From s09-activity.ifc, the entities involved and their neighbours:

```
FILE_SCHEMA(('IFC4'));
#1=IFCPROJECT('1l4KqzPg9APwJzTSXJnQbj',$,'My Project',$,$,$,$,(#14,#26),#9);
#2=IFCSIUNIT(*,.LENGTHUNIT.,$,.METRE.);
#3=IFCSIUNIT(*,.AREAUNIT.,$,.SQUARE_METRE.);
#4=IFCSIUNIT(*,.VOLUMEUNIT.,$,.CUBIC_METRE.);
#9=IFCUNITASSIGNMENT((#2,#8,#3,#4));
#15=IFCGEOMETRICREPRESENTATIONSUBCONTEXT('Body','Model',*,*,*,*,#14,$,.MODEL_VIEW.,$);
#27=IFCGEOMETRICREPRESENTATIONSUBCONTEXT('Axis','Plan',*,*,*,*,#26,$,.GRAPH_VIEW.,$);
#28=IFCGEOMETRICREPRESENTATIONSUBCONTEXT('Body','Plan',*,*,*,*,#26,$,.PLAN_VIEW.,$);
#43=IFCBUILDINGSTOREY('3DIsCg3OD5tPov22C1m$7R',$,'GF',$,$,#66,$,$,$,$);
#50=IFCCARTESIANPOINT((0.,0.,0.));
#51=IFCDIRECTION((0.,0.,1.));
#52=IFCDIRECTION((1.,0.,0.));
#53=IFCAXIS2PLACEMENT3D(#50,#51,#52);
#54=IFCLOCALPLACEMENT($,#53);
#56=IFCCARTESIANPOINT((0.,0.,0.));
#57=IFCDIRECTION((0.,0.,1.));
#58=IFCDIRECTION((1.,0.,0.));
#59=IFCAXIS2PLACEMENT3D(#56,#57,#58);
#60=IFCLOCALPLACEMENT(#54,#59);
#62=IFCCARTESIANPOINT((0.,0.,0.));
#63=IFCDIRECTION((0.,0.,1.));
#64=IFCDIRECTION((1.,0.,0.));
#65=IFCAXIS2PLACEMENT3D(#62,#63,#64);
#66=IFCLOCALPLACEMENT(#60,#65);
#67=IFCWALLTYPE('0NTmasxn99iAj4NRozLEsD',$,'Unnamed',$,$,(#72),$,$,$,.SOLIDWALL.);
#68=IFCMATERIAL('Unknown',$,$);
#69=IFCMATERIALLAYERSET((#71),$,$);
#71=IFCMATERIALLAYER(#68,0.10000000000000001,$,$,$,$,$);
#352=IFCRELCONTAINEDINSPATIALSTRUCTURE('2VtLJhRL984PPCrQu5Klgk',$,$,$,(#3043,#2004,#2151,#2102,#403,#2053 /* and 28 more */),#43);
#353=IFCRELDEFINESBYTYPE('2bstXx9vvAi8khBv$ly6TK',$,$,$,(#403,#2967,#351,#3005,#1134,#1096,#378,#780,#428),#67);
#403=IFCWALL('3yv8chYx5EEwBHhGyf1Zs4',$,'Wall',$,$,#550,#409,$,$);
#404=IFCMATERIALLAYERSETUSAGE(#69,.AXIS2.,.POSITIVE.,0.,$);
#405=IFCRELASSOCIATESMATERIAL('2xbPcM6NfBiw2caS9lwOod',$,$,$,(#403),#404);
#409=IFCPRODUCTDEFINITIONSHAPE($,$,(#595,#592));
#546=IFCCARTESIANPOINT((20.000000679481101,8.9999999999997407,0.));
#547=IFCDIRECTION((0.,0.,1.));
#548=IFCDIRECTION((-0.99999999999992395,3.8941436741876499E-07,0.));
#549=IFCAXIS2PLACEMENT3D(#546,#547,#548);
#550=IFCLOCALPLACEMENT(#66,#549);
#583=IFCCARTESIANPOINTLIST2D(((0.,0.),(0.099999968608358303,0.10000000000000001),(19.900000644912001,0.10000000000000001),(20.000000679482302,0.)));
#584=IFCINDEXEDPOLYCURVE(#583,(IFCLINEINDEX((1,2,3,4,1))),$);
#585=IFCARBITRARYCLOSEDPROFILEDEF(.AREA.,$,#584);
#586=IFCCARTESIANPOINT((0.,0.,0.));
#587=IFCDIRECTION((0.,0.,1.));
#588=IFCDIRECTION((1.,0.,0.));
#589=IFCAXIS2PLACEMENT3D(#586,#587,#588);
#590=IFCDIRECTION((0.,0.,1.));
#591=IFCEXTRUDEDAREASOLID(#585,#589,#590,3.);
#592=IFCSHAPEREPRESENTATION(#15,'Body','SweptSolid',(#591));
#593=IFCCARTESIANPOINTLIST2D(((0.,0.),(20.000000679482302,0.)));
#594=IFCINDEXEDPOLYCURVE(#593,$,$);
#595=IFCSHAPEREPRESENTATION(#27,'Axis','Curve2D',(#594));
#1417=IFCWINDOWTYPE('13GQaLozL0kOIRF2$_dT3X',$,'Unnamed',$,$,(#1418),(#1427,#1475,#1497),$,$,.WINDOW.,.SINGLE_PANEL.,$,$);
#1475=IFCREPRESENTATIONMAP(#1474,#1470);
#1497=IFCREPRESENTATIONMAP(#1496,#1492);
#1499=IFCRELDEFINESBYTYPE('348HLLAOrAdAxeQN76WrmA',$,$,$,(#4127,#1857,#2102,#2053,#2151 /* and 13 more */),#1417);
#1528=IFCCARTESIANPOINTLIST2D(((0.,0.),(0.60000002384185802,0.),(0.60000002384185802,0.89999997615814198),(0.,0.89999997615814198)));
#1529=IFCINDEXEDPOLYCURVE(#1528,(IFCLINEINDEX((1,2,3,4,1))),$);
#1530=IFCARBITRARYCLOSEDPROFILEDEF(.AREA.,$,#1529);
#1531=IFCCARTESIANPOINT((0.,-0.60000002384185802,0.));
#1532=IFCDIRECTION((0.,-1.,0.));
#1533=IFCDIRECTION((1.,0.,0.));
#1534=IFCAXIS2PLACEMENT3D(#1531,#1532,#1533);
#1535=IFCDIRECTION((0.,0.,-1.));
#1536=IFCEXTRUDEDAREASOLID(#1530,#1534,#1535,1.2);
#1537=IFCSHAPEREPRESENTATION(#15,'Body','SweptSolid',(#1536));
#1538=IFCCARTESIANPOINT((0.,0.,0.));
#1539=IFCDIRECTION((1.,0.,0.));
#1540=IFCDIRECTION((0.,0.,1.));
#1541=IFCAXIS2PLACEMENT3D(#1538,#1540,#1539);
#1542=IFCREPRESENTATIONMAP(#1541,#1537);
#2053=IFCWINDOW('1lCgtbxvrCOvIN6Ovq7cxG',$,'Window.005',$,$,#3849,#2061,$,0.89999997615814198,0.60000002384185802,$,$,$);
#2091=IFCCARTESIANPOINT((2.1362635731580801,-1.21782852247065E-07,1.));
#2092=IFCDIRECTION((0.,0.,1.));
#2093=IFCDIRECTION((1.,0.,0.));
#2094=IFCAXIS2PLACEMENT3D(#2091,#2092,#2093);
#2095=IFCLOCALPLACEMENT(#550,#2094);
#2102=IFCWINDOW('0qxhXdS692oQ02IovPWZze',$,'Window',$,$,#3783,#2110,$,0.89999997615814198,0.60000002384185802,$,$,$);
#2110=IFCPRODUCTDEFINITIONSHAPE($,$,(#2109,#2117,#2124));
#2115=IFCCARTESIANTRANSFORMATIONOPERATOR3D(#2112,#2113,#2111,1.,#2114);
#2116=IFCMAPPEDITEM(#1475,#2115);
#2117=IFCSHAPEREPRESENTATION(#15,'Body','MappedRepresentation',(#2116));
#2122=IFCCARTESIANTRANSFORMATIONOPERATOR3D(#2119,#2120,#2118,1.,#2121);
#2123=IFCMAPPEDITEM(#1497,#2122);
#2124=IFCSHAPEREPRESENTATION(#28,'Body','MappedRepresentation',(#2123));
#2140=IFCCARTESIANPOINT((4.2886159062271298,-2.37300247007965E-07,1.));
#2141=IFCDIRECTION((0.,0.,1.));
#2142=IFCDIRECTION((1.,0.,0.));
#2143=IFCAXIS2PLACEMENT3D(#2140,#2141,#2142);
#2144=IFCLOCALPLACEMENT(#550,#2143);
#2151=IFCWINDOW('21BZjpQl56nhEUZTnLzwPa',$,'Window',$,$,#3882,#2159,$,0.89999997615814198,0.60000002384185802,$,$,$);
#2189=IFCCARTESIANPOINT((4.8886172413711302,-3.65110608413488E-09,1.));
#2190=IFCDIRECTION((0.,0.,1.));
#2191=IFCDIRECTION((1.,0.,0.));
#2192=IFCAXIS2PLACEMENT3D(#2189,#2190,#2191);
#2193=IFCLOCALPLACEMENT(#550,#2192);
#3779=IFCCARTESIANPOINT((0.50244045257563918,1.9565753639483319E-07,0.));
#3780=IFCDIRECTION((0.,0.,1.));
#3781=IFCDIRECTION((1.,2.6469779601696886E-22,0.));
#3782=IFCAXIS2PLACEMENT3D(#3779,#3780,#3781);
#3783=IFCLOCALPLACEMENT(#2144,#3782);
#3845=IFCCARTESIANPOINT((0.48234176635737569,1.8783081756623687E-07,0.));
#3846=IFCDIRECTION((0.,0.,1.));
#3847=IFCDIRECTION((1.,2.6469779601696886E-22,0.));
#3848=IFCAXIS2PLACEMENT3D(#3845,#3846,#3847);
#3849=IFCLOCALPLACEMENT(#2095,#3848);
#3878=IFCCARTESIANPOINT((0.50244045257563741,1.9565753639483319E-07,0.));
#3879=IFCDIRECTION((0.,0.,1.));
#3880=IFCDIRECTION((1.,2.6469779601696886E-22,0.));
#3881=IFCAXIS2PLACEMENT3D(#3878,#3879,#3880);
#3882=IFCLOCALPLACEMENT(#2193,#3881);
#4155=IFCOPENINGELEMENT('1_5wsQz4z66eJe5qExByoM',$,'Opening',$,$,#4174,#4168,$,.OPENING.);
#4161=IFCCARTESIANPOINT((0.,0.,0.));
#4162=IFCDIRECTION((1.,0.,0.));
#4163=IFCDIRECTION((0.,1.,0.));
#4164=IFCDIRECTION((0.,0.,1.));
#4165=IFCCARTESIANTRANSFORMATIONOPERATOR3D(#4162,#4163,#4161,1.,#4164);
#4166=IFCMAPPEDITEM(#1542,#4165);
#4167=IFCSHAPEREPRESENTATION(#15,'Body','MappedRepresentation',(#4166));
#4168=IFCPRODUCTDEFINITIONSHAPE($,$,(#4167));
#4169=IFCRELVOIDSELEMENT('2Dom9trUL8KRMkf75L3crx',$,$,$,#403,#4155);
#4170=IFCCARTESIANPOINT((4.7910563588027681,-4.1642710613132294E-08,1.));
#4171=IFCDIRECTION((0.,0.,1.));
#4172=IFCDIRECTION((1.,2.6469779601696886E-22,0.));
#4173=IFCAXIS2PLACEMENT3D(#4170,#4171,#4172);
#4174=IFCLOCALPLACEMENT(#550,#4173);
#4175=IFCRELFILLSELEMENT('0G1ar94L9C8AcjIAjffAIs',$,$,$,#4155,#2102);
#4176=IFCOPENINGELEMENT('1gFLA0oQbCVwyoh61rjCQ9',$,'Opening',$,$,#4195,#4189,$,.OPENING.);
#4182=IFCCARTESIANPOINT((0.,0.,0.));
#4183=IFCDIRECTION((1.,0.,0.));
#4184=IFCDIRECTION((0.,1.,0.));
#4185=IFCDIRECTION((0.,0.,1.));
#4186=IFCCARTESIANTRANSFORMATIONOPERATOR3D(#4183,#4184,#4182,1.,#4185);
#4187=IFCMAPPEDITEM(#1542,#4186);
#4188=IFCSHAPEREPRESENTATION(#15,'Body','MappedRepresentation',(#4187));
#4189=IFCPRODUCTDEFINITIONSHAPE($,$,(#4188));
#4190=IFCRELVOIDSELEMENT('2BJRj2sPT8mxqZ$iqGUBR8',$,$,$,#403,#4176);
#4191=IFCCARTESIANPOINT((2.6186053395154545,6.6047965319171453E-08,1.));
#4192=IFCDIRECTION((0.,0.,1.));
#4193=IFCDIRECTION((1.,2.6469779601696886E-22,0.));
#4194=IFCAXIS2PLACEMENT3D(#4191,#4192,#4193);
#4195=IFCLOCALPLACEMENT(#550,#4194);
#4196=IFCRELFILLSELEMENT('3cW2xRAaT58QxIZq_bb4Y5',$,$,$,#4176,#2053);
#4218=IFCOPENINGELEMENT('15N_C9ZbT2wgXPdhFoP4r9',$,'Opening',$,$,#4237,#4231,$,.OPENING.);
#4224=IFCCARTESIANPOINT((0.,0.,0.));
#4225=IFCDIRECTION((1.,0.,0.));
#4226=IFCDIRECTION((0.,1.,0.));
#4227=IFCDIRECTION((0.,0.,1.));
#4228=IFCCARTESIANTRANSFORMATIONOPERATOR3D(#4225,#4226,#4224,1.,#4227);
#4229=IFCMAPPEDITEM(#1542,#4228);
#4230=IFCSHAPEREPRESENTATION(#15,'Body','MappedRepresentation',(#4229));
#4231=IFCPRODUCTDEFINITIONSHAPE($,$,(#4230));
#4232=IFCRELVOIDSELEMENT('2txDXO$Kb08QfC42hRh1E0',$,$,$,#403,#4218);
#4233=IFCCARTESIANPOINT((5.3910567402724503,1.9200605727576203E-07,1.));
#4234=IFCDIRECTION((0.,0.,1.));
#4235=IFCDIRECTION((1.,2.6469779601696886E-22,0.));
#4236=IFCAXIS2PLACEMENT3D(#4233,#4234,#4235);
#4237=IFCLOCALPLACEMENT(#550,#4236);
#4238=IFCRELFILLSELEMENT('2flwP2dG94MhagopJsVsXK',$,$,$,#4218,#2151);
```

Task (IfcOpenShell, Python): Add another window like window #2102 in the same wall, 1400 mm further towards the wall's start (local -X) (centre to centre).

```python
import ifcopenshell
import ifcopenshell.api.feature
import ifcopenshell.api.geometry
import ifcopenshell.api.root
import ifcopenshell.geom
import ifcopenshell.util.element
import ifcopenshell.util.placement
import ifcopenshell.util.shape
import ifcopenshell.util.unit

model = ifcopenshell.open("s09-activity.ifc")
unit_scale = ifcopenshell.util.unit.calculate_unit_scale(model)
settings = ifcopenshell.geom.settings()


def volume(element):
    """Net volume in cubic metres, openings subtracted."""
    shape = ifcopenshell.geom.create_shape(settings, element)
    return ifcopenshell.util.shape.get_volume(shape.geometry)


window = model.by_guid("0qxhXdS692oQ02IovPWZze")
opening = window.FillsVoids[0].RelatingOpeningElement
wall = opening.VoidsElements[0].RelatingBuildingElement
before = volume(wall)
shift = ifcopenshell.util.placement.get_local_placement(wall.ObjectPlacement)[:3, 0] * -1.4 / unit_scale

# copy_class copies the void relationship, type, container and properties, but no geometry.
new_opening = ifcopenshell.api.root.copy_class(model, product=opening)
new_opening.Representation = ifcopenshell.util.element.copy_deep(
    model, opening.Representation, exclude=["IfcGeometricRepresentationContext", "IfcRepresentationMap"]
)
new_window = ifcopenshell.api.root.copy_class(model, product=window)
new_window.Representation = ifcopenshell.util.element.copy_deep(
    model, window.Representation, exclude=["IfcGeometricRepresentationContext", "IfcRepresentationMap"]
)
ifcopenshell.api.feature.add_filling(model, opening=new_opening, element=new_window)

for old, new in ((opening, new_opening), (window, new_window)):
    matrix = ifcopenshell.util.placement.get_local_placement(old.ObjectPlacement)
    matrix[:3, 3] += shift
    ifcopenshell.api.geometry.edit_object_placement(model, product=new, matrix=matrix, is_si=False)

after = volume(wall)

print(f"wall volume {before:.3f} -> {after:.3f} m3")

model.write("s09-activity-out.ifc")
```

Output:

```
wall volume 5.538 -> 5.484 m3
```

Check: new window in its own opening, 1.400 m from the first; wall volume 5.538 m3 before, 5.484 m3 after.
